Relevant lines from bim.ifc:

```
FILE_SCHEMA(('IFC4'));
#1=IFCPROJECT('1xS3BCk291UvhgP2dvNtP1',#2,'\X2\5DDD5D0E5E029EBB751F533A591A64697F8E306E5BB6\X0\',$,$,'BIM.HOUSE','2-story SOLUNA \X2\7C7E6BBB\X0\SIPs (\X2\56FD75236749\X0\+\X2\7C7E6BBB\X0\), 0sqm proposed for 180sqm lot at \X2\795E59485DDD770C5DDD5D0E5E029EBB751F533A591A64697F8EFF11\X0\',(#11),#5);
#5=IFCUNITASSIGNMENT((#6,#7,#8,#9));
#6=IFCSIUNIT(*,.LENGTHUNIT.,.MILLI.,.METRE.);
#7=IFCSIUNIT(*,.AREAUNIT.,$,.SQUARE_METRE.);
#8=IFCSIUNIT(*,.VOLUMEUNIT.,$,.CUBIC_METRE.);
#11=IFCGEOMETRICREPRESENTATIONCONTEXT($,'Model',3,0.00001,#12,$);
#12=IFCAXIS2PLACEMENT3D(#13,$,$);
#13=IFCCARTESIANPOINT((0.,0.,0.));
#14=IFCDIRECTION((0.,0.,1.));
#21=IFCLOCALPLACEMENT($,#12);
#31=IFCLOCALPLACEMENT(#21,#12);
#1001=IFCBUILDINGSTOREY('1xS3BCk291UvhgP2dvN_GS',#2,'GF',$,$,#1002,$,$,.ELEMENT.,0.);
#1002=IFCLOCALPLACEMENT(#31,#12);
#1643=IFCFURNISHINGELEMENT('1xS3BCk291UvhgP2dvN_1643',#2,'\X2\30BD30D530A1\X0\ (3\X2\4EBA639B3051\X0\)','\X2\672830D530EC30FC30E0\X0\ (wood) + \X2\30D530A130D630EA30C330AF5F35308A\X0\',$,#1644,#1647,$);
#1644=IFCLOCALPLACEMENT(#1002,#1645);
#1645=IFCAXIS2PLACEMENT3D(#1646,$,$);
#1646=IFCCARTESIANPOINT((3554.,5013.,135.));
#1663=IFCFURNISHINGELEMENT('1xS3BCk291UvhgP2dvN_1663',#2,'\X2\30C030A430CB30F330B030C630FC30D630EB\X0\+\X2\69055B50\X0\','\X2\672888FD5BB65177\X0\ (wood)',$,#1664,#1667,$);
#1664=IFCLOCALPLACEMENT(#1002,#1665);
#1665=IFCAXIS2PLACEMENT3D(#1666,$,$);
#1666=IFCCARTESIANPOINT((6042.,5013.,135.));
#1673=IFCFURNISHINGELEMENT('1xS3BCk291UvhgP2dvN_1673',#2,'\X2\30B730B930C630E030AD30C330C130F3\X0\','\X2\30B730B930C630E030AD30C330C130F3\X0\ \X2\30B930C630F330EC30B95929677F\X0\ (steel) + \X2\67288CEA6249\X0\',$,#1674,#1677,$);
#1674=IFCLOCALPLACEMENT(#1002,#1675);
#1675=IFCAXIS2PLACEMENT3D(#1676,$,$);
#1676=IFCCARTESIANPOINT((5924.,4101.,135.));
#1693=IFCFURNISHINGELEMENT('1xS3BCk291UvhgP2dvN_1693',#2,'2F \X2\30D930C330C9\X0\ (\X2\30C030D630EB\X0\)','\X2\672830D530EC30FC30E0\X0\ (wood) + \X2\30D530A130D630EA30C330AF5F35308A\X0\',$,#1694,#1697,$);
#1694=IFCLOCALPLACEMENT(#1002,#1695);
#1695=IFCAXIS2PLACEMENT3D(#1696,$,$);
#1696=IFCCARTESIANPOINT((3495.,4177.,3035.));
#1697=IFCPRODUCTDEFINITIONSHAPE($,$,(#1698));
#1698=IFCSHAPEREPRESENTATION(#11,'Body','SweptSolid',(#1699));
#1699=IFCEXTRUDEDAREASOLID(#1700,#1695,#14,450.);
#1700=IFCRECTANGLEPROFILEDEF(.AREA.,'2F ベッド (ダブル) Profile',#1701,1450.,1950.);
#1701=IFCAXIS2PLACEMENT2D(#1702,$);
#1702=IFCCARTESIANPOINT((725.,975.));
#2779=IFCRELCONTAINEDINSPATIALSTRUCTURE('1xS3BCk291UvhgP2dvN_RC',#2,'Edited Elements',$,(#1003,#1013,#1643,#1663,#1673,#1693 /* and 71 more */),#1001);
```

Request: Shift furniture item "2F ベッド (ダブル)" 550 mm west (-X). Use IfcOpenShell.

```python
import ifcopenshell
import ifcopenshell.api.geometry
import ifcopenshell.util.placement
import ifcopenshell.util.unit

model = ifcopenshell.open("bim.ifc")
unit_scale = ifcopenshell.util.unit.calculate_unit_scale(model)

item = model.by_guid("1xS3BCk291UvhgP2dvN_1693")
matrix = ifcopenshell.util.placement.get_local_placement(item.ObjectPlacement)
matrix[0, 3] -= 0.55 / unit_scale
ifcopenshell.api.geometry.edit_object_placement(model, product=item, matrix=matrix, is_si=False)

print(ifcopenshell.util.placement.get_local_placement(item.ObjectPlacement).round(3) + 0.0)

model.write("bim_rev.ifc")
```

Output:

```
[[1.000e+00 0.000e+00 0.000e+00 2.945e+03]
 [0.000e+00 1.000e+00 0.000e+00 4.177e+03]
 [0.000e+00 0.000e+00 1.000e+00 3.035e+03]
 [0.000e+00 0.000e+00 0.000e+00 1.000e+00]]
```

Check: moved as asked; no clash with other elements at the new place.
